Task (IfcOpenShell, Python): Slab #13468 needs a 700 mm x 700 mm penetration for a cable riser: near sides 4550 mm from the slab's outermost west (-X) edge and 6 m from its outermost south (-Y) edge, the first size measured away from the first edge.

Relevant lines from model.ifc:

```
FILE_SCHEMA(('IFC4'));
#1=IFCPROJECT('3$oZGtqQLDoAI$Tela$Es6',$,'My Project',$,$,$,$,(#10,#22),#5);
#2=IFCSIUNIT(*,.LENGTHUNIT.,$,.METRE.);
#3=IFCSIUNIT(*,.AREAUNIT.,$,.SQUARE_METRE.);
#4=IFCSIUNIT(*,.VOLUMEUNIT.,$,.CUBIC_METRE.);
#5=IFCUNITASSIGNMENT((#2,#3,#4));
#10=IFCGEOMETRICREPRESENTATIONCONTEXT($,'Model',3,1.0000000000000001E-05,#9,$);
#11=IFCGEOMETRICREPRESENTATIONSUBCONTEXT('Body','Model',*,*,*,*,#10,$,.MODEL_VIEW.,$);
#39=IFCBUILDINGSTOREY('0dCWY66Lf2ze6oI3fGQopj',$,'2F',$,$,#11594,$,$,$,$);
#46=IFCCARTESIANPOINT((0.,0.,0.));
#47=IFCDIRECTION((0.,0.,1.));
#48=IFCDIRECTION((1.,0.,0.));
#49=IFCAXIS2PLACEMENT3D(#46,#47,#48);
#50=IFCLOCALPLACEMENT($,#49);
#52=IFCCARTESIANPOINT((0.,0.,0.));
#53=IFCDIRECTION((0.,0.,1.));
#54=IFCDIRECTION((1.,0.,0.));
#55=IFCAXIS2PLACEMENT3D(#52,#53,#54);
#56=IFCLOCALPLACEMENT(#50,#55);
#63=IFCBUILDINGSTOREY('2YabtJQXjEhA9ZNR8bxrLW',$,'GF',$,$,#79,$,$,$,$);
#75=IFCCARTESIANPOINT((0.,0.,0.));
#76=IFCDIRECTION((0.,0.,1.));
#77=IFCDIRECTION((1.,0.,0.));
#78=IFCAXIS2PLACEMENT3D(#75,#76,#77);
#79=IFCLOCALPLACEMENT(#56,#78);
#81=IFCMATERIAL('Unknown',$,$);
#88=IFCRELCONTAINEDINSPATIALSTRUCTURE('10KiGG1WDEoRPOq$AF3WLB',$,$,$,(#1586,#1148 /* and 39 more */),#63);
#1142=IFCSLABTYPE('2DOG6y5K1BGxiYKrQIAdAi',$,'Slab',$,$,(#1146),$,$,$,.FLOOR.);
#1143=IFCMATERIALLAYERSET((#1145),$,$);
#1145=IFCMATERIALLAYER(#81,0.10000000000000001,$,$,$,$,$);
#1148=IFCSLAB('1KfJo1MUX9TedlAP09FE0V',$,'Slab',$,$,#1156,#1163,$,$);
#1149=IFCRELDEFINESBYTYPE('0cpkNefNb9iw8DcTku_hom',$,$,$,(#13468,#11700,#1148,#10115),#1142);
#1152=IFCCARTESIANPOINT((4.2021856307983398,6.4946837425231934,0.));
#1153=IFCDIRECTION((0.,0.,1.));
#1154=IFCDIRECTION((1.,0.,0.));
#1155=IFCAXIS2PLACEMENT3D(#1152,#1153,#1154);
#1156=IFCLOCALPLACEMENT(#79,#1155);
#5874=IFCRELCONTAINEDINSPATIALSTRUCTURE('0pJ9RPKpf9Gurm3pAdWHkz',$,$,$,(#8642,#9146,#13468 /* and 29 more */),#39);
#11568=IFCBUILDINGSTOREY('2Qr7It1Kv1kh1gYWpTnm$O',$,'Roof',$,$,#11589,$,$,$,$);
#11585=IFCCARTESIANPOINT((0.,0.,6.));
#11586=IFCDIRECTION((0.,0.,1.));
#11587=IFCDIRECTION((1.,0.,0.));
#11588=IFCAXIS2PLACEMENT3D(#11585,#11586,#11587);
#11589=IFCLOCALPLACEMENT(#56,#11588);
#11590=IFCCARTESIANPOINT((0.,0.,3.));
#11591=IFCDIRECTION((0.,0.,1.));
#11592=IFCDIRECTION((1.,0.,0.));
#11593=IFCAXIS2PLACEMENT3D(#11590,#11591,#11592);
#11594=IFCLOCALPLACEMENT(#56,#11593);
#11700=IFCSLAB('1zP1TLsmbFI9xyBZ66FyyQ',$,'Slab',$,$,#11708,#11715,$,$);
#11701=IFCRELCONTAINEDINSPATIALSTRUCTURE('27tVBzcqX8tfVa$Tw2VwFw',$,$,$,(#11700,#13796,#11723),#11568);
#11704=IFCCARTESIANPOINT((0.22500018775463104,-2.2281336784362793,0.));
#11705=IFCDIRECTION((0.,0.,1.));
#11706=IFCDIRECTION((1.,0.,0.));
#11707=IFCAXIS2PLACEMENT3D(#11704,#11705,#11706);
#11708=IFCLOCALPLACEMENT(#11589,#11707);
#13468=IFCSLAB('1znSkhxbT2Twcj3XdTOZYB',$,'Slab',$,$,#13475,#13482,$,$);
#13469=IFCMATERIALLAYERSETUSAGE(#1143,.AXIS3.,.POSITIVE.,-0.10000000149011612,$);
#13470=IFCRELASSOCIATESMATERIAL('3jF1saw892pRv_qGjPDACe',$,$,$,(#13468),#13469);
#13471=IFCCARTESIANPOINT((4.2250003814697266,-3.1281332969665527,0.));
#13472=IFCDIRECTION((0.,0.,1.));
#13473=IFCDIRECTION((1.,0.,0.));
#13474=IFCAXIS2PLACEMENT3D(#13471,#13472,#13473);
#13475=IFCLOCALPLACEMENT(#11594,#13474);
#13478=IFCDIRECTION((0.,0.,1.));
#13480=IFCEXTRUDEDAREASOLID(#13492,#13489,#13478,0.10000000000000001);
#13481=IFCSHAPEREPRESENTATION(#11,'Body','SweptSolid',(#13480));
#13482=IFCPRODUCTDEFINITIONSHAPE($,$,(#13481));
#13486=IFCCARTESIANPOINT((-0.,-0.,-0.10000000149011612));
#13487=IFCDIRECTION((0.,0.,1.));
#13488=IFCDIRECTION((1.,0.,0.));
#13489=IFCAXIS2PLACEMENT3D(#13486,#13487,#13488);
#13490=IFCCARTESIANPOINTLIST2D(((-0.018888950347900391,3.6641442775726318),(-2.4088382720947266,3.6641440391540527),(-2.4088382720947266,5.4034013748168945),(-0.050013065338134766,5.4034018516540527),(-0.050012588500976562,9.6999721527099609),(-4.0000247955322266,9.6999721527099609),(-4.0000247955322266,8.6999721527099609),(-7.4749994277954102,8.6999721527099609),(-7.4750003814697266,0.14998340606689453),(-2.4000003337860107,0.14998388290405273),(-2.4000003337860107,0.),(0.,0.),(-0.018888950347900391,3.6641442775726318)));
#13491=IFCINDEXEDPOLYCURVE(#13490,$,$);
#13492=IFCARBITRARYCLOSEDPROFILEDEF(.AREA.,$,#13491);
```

```python
import numpy as np
import ifcopenshell
import ifcopenshell.api.feature
import ifcopenshell.api.geometry
import ifcopenshell.api.root
import ifcopenshell.geom
import ifcopenshell.util.placement
import ifcopenshell.util.representation
import ifcopenshell.util.shape
import ifcopenshell.util.unit

model = ifcopenshell.open("model.ifc")
unit_scale = ifcopenshell.util.unit.calculate_unit_scale(model)
settings = ifcopenshell.geom.settings()


def volume(element):
    """Net volume in cubic metres, openings subtracted."""
    shape = ifcopenshell.geom.create_shape(settings, element)
    return ifcopenshell.util.shape.get_volume(shape.geometry)


slab = model.by_id(13468)
before = volume(slab)

# Extent in the slab's own axes, in metres. The edges named are its -X and -Y sides.
slab_shape = ifcopenshell.geom.create_shape(settings, slab)
vertices = ifcopenshell.util.shape.get_vertices(slab_shape.geometry)
x_min, y_min, bottom = vertices.min(axis=0)
top = vertices[:, 2].max()

opening = ifcopenshell.api.root.create_entity(model, ifc_class="IfcOpeningElement", name="Cable riser opening", predefined_type="OPENING")
context = ifcopenshell.util.representation.get_context(model, "Model", "Body", "MODEL_VIEW")
width, depth = 0.7, 0.7
outline = [(0.0, 0.0), (width, 0.0), (width, depth), (0.0, depth), (0.0, 0.0)]
# Overshoot both faces by 50 mm so the cut is clean.
shape = ifcopenshell.api.geometry.add_slab_representation(
    model, context=context, depth=top - bottom + 0.1, polyline=outline
)
ifcopenshell.api.geometry.assign_representation(model, product=opening, representation=shape)

matrix = ifcopenshell.util.placement.get_local_placement(slab.ObjectPlacement)
matrix[:, 3] = matrix @ np.append(np.array([x_min + 4.55, y_min + 6, bottom - 0.05]) / unit_scale, 1.0)
ifcopenshell.api.geometry.edit_object_placement(model, product=opening, matrix=matrix, is_si=False)
ifcopenshell.api.feature.add_feature(model, feature=opening, element=slab)

after = volume(slab)

print(f"slab volume {before:.3f} -> {after:.3f} m3")

model.write("model-out.ifc")
```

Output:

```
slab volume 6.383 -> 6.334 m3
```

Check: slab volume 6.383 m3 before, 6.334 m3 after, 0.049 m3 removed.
